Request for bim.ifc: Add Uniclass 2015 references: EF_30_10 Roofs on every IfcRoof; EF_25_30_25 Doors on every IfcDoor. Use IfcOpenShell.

First a look at what the model holds.

```python
import ifcopenshell

model = ifcopenshell.open("bim.ifc")
print(model.schema)
print("classifications:", [c.Name for c in model.by_type("IfcClassification")])
for ifc_class in ("IfcDoor", "IfcRoof", "IfcStair", "IfcWall", "IfcWindow"):
    print(ifc_class, len(model.by_type(ifc_class)))
```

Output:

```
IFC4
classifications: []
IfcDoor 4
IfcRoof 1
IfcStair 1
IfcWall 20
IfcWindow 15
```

```python
import ifcopenshell
import ifcopenshell.api.classification

model = ifcopenshell.open("bim.ifc")

system = ifcopenshell.api.classification.add_classification(model, classification="Uniclass 2015")

codes = {
    "IfcRoof": ("EF_30_10", "Roofs"),
    "IfcDoor": ("EF_25_30_25", "Doors"),
}
for ifc_class, (code, name) in codes.items():
    products = model.by_type(ifc_class)
    ifcopenshell.api.classification.add_reference(
        model, products=products, classification=system, identification=code, name=name
    )
    print(code, len(products))

model.write("bim_edited.ifc")
```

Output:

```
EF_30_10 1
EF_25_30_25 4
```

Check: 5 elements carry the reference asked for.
